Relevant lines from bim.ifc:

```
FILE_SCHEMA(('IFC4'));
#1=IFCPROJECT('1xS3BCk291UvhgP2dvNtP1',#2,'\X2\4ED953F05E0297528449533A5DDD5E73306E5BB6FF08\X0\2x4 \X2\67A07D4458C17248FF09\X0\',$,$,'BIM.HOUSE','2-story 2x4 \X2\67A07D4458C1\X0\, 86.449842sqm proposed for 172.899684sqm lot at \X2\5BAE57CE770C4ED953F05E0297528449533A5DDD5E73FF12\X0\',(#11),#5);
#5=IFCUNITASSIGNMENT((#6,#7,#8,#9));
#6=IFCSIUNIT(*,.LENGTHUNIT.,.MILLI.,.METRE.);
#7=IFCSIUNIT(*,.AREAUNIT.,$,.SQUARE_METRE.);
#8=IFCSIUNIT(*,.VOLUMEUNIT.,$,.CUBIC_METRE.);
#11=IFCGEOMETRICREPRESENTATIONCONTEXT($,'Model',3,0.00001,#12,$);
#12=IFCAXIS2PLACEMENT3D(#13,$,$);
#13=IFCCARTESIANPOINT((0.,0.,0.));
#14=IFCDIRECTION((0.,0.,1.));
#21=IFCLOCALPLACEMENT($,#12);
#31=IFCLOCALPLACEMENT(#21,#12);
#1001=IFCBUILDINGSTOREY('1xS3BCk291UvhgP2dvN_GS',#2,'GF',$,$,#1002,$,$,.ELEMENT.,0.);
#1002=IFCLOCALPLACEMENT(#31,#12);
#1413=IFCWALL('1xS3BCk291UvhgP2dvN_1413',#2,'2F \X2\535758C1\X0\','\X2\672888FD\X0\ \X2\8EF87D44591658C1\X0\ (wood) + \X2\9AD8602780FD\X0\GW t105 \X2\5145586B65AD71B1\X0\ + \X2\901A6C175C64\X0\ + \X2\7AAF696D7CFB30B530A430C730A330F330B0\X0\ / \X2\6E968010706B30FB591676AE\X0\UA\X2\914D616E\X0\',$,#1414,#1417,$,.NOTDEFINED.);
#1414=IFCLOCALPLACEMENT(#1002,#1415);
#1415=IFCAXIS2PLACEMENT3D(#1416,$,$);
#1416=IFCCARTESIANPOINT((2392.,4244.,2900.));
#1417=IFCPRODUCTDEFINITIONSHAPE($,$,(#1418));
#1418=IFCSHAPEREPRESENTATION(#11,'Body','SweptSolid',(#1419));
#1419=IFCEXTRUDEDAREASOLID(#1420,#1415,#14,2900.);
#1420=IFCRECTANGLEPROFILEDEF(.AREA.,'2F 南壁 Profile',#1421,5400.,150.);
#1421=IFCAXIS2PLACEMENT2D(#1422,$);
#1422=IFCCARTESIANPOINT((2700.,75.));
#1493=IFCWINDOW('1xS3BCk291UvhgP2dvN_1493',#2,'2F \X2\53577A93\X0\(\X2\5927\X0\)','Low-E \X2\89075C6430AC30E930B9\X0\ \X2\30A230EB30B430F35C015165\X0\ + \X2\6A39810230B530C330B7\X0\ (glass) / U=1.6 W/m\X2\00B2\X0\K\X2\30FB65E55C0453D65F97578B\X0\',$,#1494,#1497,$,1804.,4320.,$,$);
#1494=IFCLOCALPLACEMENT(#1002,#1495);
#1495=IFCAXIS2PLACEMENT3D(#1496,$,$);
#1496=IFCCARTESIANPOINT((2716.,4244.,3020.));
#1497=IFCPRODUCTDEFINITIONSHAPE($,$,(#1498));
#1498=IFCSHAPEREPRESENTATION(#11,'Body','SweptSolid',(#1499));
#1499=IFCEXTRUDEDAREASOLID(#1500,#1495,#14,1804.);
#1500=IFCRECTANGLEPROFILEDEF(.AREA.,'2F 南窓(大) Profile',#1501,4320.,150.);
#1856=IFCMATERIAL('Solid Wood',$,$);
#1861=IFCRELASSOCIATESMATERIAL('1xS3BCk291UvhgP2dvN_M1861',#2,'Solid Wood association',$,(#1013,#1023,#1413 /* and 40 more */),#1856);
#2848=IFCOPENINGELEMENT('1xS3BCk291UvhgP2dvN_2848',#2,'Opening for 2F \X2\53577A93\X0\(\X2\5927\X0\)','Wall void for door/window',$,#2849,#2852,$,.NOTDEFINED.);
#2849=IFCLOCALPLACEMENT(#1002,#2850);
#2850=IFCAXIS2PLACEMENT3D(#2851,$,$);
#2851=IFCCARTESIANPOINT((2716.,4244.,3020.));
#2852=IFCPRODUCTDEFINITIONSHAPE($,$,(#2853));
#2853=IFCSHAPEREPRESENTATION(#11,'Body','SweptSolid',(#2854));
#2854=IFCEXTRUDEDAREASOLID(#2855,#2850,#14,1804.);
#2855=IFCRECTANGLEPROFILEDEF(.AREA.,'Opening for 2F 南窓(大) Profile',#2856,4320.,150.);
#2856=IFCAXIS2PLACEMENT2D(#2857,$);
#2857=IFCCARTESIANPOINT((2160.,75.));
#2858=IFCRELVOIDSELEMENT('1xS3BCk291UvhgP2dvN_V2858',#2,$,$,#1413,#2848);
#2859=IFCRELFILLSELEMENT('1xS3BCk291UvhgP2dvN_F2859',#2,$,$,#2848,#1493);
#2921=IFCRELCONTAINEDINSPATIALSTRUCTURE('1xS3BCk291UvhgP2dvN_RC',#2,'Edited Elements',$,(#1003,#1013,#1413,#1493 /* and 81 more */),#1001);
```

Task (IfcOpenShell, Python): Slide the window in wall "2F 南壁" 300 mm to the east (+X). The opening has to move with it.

```python
import ifcopenshell
import ifcopenshell.api.geometry
import ifcopenshell.util.placement
import ifcopenshell.util.unit

model = ifcopenshell.open("bim.ifc")
unit_scale = ifcopenshell.util.unit.calculate_unit_scale(model)

window = model.by_guid("1xS3BCk291UvhgP2dvN_1493")
opening = window.FillsVoids[0].RelatingOpeningElement
wall = opening.VoidsElements[0].RelatingBuildingElement

wall_matrix = ifcopenshell.util.placement.get_local_placement(wall.ObjectPlacement)
shift = wall_matrix[:3, 0] * 0.3 / unit_scale
before = ifcopenshell.util.placement.get_local_placement(window.ObjectPlacement)[:3, 3].copy()

# The window is not placed relative to its opening, so move both.
for product in (opening, window):
    matrix = ifcopenshell.util.placement.get_local_placement(product.ObjectPlacement)
    matrix[:3, 3] += shift
    ifcopenshell.api.geometry.edit_object_placement(model, product=product, matrix=matrix, is_si=False)

after = ifcopenshell.util.placement.get_local_placement(window.ObjectPlacement)[:3, 3]
print("window moved by", (after - before).round(3) + 0.0)

model.write("bim_updated.ifc")
```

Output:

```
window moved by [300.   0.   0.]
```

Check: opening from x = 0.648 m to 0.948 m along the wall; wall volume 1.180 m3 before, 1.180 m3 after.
